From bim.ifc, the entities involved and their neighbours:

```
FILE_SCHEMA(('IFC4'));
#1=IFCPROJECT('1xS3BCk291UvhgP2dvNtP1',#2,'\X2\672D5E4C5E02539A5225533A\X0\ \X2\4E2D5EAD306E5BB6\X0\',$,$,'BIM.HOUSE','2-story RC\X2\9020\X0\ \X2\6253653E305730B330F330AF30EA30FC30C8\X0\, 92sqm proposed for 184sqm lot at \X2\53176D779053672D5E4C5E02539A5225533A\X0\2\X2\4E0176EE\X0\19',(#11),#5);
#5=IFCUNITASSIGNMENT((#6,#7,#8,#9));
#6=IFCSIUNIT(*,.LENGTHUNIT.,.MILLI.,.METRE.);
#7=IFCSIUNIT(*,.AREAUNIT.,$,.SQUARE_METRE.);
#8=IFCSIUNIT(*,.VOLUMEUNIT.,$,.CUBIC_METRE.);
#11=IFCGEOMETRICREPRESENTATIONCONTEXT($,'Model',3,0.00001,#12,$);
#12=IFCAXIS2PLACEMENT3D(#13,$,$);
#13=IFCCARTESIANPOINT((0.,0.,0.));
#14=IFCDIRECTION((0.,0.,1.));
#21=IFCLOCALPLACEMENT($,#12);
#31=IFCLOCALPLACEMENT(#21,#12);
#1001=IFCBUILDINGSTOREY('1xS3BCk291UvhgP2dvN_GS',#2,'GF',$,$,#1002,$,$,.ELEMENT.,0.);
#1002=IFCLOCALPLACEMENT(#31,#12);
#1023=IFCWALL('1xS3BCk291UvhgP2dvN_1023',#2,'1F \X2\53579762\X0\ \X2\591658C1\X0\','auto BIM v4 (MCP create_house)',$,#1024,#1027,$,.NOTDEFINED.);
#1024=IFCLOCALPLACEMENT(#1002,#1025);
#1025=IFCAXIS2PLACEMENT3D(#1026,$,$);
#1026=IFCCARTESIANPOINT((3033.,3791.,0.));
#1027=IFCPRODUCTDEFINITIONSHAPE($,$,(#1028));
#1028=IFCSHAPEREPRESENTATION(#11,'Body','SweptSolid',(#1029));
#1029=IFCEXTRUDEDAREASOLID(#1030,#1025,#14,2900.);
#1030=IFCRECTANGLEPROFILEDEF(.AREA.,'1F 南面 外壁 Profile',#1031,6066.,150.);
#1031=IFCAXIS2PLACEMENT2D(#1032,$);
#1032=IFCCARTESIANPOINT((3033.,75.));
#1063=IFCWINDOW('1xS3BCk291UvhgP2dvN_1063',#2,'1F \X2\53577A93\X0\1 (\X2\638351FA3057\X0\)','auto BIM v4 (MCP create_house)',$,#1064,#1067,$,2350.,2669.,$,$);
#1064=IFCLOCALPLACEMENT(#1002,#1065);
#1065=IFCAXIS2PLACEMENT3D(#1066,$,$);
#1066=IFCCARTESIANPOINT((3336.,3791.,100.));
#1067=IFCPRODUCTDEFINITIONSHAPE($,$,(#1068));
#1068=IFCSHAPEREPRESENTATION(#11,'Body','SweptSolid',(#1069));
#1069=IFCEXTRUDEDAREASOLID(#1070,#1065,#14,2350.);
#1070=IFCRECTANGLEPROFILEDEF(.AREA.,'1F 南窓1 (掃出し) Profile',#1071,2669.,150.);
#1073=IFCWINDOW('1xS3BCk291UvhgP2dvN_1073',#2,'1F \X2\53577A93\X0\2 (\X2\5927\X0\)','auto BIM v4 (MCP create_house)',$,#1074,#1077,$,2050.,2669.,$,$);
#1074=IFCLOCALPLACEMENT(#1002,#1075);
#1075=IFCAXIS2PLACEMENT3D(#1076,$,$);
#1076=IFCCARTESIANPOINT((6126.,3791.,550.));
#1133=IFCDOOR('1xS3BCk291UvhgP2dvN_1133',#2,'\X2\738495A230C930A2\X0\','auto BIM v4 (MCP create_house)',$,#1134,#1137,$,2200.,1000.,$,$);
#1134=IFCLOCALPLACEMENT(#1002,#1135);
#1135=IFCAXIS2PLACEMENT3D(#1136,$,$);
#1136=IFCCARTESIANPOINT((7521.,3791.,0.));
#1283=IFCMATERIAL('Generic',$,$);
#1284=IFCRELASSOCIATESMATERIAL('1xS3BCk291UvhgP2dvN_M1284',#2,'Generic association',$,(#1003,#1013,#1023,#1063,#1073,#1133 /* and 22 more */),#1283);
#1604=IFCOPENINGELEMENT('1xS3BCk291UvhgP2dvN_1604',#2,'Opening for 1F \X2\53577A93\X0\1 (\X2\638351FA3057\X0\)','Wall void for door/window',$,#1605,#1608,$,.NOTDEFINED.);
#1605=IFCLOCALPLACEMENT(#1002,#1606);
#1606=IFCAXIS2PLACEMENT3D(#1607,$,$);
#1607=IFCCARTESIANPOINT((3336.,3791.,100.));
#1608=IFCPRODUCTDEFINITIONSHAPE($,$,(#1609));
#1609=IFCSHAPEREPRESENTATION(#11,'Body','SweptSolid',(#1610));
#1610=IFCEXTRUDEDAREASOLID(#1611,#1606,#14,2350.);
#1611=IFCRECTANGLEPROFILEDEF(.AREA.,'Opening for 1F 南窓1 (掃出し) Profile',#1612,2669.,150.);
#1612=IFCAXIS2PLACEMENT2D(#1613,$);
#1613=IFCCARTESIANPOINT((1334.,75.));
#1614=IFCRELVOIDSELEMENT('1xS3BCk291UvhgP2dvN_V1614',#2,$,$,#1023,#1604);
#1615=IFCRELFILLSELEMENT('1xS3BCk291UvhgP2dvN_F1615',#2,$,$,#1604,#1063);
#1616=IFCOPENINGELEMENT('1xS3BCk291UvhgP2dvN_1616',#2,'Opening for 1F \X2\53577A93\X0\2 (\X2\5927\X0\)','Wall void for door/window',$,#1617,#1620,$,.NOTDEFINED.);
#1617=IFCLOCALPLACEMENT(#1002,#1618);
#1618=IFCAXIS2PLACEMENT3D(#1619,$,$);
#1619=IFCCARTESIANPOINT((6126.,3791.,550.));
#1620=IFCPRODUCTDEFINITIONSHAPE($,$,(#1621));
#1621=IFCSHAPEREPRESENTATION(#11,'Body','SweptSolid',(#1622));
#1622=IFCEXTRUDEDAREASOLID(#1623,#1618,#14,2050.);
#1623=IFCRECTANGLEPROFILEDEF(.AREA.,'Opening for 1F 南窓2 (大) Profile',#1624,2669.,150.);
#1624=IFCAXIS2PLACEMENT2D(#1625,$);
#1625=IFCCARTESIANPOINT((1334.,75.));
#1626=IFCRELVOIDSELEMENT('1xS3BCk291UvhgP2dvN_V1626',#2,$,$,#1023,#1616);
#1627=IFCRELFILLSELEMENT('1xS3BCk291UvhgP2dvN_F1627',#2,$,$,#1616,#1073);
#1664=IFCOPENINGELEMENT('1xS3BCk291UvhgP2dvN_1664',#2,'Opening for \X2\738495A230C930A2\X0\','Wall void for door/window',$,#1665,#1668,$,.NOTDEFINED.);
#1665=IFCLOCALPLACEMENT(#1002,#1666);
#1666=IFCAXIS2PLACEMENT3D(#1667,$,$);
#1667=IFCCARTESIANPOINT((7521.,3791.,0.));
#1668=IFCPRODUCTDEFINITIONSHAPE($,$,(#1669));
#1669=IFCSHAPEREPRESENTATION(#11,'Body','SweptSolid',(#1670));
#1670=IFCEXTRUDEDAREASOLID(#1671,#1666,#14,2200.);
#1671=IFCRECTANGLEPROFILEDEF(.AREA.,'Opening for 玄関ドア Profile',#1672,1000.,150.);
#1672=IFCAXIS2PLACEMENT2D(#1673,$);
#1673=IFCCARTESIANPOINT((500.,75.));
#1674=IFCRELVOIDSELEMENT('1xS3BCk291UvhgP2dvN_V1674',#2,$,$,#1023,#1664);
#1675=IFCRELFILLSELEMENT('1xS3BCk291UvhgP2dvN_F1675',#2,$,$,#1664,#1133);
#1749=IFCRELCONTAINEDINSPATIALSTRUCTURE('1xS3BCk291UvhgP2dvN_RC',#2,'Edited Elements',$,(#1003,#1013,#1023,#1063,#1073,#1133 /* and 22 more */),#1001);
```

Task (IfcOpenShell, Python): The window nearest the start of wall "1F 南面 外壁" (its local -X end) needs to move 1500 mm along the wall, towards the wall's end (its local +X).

```python
import ifcopenshell
import ifcopenshell.api.geometry
import ifcopenshell.util.placement

model = ifcopenshell.open("bim.ifc")

window = model.by_guid("1xS3BCk291UvhgP2dvN_1063")
opening = window.FillsVoids[0].RelatingOpeningElement
wall = opening.VoidsElements[0].RelatingBuildingElement

wall_matrix = ifcopenshell.util.placement.get_local_placement(wall.ObjectPlacement)
shift = wall_matrix[:3, 0] * 1500.0
before = ifcopenshell.util.placement.get_local_placement(window.ObjectPlacement)[:3, 3].copy()

# The window is not placed relative to its opening, so move both.
for product in (opening, window):
    matrix = ifcopenshell.util.placement.get_local_placement(product.ObjectPlacement)
    matrix[:3, 3] += shift
    ifcopenshell.api.geometry.edit_object_placement(model, product=product, matrix=matrix, is_si=False)

after = ifcopenshell.util.placement.get_local_placement(window.ObjectPlacement)[:3, 3]
print("window moved by", (after - before).round(3) + 0.0)

model.write("bim_rev.ifc")
```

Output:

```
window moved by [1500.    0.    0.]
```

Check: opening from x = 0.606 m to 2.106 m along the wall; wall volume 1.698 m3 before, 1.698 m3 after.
